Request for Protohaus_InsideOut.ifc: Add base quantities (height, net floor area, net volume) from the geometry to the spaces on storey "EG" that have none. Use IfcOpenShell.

First a look at what the model holds.

```python
import ifcopenshell
import ifcopenshell.util.element
import ifcopenshell.util.unit

model = ifcopenshell.open("Protohaus_InsideOut.ifc")
print(model.schema)
for unit_type in ("LENGTHUNIT", "AREAUNIT", "VOLUMEUNIT"):
    print(unit_type, ifcopenshell.util.unit.calculate_unit_scale(model, unit_type))
storey = next(s for s in model.by_type("IfcBuildingStorey") if s.Name == "EG")
spaces = [e for e in ifcopenshell.util.element.get_decomposition(storey) if e.is_a("IfcSpace")]
for e in sorted(spaces, key=lambda e: e.id()):
    print(e.id(), e.is_a(), e.Name, list(ifcopenshell.util.element.get_psets(e, qtos_only=True)), sep=" | ")
```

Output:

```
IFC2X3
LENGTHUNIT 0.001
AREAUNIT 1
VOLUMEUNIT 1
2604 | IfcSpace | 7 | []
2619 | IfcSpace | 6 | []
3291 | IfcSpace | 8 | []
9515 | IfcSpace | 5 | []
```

```python
import ifcopenshell
import ifcopenshell.api.pset
import ifcopenshell.geom
import ifcopenshell.util.element
import ifcopenshell.util.shape
import ifcopenshell.util.unit

model = ifcopenshell.open("Protohaus_InsideOut.ifc")
unit_scale = ifcopenshell.util.unit.calculate_unit_scale(model)
area_scale = ifcopenshell.util.unit.calculate_unit_scale(model, "AREAUNIT")
volume_scale = ifcopenshell.util.unit.calculate_unit_scale(model, "VOLUMEUNIT")
settings = ifcopenshell.geom.settings()

storey = next(s for s in model.by_type("IfcBuildingStorey") if s.Name == "EG")
spaces = [e for e in ifcopenshell.util.element.get_decomposition(storey) if e.is_a("IfcSpace")]

for e in sorted(spaces, key=lambda e: e.id()):
    if ifcopenshell.util.element.get_psets(e, qtos_only=True, should_inherit=False):
        continue
    # Geometry comes back in metres, in the element's own axes.
    shape = ifcopenshell.geom.create_shape(settings, e)
    values = {
        "Height": ifcopenshell.util.shape.get_z(shape.geometry) / unit_scale,
        "NetFloorArea": ifcopenshell.util.shape.get_footprint_area(shape.geometry) / area_scale,
        "NetVolume": ifcopenshell.util.shape.get_volume(shape.geometry) / volume_scale,
    }
    qto = ifcopenshell.api.pset.add_qto(model, product=e, name="BaseQuantities")
    ifcopenshell.api.pset.edit_qto(model, qto=qto, properties=values)
    print(e.id(), {k: round(v, 3) for k, v in values.items()})

model.write("Protohaus_InsideOut_v2.ifc")
```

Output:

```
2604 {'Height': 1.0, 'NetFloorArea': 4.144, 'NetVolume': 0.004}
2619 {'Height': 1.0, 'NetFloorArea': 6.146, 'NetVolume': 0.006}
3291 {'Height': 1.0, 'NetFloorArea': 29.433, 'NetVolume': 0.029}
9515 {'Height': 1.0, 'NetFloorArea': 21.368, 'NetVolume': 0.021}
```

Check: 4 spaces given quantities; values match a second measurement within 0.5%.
